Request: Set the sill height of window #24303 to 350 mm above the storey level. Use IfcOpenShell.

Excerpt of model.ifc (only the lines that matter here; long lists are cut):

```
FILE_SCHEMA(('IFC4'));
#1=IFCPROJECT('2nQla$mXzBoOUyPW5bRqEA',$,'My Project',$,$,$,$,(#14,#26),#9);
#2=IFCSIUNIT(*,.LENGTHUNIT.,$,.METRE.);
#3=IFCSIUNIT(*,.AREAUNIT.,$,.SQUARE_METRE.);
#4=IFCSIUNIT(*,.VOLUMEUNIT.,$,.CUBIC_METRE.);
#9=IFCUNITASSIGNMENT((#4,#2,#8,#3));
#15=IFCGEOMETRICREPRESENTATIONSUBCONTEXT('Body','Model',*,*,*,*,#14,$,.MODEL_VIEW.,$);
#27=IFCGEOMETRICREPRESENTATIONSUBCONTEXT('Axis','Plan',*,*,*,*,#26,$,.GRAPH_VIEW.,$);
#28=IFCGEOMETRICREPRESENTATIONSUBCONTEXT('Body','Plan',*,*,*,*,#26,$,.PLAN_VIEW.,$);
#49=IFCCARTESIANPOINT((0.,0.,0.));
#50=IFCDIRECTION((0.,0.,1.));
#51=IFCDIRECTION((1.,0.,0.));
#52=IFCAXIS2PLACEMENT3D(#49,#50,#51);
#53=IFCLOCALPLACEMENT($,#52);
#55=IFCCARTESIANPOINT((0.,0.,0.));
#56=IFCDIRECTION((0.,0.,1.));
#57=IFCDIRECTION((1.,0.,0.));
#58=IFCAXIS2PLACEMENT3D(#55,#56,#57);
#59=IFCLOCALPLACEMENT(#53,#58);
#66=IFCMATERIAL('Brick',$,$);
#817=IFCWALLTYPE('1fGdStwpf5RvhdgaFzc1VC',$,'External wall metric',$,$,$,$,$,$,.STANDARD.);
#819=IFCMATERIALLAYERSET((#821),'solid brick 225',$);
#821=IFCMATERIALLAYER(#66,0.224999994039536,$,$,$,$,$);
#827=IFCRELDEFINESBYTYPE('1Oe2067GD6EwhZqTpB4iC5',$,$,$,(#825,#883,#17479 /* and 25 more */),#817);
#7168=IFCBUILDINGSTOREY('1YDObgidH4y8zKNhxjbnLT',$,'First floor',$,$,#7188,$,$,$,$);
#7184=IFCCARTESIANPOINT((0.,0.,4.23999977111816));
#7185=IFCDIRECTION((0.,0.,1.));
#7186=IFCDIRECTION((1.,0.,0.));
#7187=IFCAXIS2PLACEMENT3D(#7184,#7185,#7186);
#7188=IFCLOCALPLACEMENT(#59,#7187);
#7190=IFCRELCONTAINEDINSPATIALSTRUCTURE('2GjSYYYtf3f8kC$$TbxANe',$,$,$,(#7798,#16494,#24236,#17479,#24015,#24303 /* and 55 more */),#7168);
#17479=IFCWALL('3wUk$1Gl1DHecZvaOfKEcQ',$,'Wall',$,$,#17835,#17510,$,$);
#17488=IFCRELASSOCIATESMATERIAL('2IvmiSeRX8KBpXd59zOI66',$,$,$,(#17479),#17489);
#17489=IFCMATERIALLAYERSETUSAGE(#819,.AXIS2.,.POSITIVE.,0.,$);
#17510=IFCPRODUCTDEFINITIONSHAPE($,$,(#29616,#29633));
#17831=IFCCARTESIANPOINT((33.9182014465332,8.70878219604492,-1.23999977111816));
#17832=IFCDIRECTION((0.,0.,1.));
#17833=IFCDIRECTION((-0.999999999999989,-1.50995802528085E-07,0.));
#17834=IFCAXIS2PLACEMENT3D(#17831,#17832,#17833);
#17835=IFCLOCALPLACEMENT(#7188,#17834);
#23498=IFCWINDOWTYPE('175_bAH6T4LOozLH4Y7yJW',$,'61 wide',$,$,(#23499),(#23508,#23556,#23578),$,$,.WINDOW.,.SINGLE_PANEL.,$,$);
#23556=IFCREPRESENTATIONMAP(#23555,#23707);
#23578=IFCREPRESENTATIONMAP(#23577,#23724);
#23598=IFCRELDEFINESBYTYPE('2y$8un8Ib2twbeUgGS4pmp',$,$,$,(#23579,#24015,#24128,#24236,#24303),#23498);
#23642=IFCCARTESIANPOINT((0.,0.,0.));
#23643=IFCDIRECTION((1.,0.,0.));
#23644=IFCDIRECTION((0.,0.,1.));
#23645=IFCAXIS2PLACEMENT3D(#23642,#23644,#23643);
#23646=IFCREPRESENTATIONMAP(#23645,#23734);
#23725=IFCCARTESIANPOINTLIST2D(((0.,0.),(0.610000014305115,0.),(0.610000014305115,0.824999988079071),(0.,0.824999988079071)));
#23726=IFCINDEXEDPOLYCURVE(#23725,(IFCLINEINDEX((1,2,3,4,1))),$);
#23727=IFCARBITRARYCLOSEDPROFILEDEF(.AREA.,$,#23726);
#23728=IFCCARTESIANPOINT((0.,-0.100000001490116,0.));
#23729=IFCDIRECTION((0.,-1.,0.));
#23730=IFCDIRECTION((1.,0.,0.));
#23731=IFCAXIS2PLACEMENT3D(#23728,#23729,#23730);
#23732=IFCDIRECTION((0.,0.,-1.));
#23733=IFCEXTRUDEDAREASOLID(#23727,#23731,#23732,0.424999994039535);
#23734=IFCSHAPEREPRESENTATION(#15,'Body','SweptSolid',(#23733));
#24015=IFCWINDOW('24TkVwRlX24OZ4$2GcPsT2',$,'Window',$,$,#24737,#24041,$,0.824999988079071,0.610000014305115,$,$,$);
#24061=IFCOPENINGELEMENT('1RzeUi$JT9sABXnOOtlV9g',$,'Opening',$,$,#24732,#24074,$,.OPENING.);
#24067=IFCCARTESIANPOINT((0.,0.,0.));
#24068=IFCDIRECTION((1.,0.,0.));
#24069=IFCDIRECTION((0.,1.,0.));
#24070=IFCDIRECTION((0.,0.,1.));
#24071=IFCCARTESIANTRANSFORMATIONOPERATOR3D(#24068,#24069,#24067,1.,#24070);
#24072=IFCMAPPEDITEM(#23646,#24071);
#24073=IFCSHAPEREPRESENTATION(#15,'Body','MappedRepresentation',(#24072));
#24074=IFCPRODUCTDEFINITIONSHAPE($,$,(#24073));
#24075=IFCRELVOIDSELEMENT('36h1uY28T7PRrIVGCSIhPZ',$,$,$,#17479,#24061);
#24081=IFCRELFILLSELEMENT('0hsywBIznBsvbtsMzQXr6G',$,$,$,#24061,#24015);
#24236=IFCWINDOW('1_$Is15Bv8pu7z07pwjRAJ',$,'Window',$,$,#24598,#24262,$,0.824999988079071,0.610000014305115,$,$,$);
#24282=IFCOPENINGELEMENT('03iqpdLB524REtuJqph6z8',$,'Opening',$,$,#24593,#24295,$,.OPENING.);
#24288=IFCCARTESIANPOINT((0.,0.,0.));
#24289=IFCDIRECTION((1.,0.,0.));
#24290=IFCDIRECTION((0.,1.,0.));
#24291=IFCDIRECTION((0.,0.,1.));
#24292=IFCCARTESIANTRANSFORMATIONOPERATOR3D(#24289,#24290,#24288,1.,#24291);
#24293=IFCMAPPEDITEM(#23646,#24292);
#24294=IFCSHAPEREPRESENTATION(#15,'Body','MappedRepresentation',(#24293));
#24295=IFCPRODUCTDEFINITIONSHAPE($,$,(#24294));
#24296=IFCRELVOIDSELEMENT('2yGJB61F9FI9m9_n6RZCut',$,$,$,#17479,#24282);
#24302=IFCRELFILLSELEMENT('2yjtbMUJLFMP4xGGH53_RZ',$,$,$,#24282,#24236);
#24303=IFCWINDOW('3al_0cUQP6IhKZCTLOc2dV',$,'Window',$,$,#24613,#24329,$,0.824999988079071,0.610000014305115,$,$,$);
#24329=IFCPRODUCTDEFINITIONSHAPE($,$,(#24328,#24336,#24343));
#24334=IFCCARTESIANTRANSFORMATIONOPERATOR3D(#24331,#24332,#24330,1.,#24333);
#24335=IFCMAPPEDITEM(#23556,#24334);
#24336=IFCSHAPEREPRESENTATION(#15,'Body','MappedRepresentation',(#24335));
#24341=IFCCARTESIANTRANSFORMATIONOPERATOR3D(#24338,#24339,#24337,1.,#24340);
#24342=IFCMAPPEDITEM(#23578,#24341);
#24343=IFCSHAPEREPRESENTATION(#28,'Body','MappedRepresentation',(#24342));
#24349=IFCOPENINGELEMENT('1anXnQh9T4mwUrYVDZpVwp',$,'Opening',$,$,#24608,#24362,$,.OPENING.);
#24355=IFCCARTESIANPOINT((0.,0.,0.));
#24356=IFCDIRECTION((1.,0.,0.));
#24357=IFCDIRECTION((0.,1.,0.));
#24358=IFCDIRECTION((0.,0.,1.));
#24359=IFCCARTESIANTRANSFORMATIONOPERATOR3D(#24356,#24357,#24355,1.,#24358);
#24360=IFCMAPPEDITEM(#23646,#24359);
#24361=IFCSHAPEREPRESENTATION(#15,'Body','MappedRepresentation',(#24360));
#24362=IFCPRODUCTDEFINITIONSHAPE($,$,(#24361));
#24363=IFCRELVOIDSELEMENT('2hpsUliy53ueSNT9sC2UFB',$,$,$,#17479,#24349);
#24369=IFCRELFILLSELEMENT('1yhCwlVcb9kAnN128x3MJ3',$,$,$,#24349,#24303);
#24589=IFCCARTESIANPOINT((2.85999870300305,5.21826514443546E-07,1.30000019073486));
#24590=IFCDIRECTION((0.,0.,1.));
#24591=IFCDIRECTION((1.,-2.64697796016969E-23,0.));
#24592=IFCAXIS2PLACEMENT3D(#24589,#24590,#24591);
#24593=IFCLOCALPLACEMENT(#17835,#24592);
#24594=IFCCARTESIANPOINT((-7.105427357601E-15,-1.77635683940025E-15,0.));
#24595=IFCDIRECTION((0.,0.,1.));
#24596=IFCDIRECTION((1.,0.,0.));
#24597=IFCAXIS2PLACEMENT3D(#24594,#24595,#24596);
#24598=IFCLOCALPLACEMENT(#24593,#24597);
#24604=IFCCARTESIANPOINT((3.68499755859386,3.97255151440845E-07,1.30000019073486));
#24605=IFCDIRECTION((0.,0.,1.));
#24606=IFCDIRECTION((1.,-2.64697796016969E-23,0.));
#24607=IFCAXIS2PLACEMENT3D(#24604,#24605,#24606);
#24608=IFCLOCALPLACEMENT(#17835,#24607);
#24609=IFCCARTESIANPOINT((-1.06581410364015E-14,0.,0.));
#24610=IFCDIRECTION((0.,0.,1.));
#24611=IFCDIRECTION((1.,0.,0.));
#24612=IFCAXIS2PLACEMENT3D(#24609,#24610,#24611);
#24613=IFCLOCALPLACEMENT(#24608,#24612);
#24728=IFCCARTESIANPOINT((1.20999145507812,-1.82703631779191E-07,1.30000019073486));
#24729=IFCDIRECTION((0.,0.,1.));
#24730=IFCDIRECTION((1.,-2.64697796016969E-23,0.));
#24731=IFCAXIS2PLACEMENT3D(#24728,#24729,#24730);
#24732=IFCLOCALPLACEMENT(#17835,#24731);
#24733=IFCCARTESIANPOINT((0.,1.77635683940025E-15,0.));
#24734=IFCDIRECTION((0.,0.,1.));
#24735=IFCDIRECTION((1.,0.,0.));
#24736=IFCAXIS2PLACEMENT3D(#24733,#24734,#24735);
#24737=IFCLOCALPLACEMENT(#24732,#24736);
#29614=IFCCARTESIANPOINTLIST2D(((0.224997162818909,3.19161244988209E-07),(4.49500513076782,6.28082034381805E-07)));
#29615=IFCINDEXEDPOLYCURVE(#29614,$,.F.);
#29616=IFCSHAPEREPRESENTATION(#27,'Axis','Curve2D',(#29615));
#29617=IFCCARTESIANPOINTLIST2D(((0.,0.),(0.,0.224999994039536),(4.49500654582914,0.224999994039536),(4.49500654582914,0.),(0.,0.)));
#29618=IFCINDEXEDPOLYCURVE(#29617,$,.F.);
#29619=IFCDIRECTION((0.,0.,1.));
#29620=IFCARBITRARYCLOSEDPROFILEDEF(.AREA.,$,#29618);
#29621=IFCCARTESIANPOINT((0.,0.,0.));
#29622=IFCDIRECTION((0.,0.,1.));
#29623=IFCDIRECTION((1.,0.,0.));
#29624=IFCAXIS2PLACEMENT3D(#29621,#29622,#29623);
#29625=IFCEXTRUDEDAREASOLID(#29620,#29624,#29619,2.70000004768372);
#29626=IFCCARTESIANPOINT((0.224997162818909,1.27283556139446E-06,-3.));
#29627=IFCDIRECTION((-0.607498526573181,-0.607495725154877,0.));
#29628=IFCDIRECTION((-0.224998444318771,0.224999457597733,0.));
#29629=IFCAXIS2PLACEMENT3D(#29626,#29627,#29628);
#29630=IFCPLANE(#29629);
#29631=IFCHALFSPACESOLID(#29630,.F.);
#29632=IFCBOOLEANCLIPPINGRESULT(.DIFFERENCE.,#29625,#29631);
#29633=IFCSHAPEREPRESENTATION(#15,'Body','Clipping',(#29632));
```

```python
import numpy as np
import ifcopenshell
import ifcopenshell.api.geometry
import ifcopenshell.geom
import ifcopenshell.util.element
import ifcopenshell.util.placement
import ifcopenshell.util.shape
import ifcopenshell.util.unit

model = ifcopenshell.open("model.ifc")
unit_scale = ifcopenshell.util.unit.calculate_unit_scale(model)

window = model.by_guid("3al_0cUQP6IhKZCTLOc2dV")
opening = window.FillsVoids[0].RelatingOpeningElement
storey = ifcopenshell.util.element.get_container(window, ifc_class="IfcBuildingStorey")
level = ifcopenshell.util.placement.get_local_placement(storey.ObjectPlacement)[2, 3]

# The opening's origin need not be at the sill, so measure its lowest point.
shape = ifcopenshell.geom.create_shape(ifcopenshell.geom.settings(), opening)
bottom = ifcopenshell.util.shape.get_shape_bottom_elevation(shape, shape.geometry) / unit_scale
dz = level + 0.35 - bottom

shift = np.array([0.0, 0.0, dz])
# The window is placed relative to its opening, so it follows when the opening moves.
matrix = ifcopenshell.util.placement.get_local_placement(opening.ObjectPlacement)
matrix[:3, 3] += shift
ifcopenshell.api.geometry.edit_object_placement(
    model, product=opening, matrix=matrix, is_si=False, should_transform_children=True
)

print(f"moved by {dz * unit_scale:+.3f} m")

model.write("model_rev.ifc")
```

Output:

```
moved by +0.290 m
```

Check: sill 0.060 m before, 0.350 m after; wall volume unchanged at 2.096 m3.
